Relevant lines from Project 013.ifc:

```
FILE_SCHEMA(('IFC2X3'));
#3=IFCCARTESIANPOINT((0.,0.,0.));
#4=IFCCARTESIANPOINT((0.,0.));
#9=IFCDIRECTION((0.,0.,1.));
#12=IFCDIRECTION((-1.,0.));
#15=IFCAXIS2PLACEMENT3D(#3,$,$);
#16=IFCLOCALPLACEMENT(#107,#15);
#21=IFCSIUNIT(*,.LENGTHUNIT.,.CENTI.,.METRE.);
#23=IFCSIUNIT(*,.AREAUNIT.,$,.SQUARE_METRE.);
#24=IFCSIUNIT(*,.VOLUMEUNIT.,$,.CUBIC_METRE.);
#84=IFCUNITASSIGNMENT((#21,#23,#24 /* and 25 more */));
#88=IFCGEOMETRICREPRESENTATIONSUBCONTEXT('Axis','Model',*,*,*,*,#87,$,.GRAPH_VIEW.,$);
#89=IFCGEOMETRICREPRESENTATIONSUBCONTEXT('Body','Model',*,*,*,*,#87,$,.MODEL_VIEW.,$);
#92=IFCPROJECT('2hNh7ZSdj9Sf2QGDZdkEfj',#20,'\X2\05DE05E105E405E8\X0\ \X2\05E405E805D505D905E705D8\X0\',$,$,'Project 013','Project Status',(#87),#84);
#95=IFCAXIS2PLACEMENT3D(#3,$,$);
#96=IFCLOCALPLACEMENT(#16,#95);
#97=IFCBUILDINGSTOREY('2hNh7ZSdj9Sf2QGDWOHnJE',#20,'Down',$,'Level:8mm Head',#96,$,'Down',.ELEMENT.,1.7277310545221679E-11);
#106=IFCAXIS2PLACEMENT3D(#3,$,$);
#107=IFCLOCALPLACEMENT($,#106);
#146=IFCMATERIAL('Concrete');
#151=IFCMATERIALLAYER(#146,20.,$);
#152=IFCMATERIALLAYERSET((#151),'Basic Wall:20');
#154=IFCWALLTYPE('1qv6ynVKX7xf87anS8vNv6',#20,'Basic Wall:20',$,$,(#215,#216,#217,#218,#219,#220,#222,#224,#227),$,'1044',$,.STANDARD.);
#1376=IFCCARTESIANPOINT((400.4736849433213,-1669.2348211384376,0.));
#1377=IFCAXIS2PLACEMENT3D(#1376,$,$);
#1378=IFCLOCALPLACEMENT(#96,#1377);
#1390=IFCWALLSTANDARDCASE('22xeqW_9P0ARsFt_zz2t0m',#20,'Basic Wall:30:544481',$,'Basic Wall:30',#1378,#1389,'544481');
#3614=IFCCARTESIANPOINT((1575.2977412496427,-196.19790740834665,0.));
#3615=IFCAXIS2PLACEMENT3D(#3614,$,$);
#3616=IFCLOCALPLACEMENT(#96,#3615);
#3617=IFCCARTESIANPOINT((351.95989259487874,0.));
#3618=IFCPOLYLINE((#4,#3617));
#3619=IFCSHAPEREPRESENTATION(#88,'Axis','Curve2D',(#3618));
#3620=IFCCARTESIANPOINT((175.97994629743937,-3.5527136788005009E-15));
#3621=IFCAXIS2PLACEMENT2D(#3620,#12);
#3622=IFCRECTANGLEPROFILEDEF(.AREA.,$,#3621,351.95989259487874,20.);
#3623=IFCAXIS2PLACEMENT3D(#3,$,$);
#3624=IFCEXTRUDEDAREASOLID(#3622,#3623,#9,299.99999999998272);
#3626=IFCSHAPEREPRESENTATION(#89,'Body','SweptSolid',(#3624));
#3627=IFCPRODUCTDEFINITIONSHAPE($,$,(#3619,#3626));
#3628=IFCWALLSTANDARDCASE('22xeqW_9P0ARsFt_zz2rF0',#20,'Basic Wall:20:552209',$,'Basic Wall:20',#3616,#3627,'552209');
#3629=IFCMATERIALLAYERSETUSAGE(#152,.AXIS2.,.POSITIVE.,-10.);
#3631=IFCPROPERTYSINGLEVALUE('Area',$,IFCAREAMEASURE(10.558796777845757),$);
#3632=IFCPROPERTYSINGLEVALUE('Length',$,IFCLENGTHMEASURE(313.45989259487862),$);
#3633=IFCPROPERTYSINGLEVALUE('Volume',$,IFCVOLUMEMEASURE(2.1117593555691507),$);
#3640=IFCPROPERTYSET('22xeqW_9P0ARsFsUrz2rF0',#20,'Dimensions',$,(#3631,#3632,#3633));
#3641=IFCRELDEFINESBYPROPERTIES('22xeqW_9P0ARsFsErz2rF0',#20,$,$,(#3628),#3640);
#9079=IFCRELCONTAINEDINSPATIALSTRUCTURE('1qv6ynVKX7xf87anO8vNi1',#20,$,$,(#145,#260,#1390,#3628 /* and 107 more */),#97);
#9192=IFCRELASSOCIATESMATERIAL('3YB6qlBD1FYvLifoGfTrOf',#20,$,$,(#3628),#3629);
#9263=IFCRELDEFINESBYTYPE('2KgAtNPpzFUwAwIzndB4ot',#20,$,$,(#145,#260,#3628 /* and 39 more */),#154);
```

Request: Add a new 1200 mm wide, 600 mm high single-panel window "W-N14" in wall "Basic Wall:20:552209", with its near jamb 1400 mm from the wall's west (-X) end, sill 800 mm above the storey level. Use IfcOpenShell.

```python
import numpy as np
import ifcopenshell
import ifcopenshell.api.feature
import ifcopenshell.api.geometry
import ifcopenshell.api.pset
import ifcopenshell.api.root
import ifcopenshell.api.spatial
import ifcopenshell.api.type
import ifcopenshell.geom
import ifcopenshell.util.element
import ifcopenshell.util.placement
import ifcopenshell.util.representation
import ifcopenshell.util.shape
import ifcopenshell.util.unit

model = ifcopenshell.open("Project 013.ifc")
unit_scale = ifcopenshell.util.unit.calculate_unit_scale(model)
area_scale = ifcopenshell.util.unit.calculate_unit_scale(model, "AREAUNIT")
volume_scale = ifcopenshell.util.unit.calculate_unit_scale(model, "VOLUMEUNIT")
settings = ifcopenshell.geom.settings()


def volume(element):
    """Net volume in cubic metres, openings subtracted."""
    shape = ifcopenshell.geom.create_shape(settings, element)
    return ifcopenshell.util.shape.get_volume(shape.geometry)


wall = model.by_guid("22xeqW_9P0ARsFt_zz2rF0")
storey = ifcopenshell.util.element.get_container(wall, ifc_class="IfcBuildingStorey")
context = ifcopenshell.util.representation.get_context(model, "Model", "Body", "MODEL_VIEW")
before = volume(wall)

width, height, from_end, sill = 1.2, 0.6, 1.4, 0.8  # metres

# The wall runs along its own X axis, and the end named is its -X end.
wall_shape = ifcopenshell.geom.create_shape(settings, wall)
x, y, z = ifcopenshell.util.shape.get_vertices(wall_shape.geometry).T
start = x.min() + from_end
face, thickness = float(y.min()), float(y.max() - y.min())
wall_matrix = ifcopenshell.util.placement.get_local_placement(wall.ObjectPlacement)
level = ifcopenshell.util.placement.get_local_placement(storey.ObjectPlacement)[2, 3]


def in_wall(x, y):
    """Placement at x, y metres in the wall's axes, at sill height."""
    matrix = wall_matrix.copy()
    matrix[:, 3] = wall_matrix @ np.array([x / unit_scale, y / unit_scale, 0.0, 1.0])
    matrix[2, 3] = level + sill / unit_scale
    return matrix


# Opening: a box that overshoots both wall faces by 50 mm.
opening = ifcopenshell.api.root.create_entity(model, ifc_class="IfcOpeningElement")
box = ifcopenshell.api.geometry.add_wall_representation(
    model, context=context, length=width, height=height, thickness=thickness + 0.1
)
ifcopenshell.api.geometry.assign_representation(model, product=opening, representation=box)
ifcopenshell.api.geometry.edit_object_placement(model, product=opening, matrix=in_wall(start, face - 0.05), is_si=False)
ifcopenshell.api.feature.add_feature(model, feature=opening, element=wall)

window = ifcopenshell.api.root.create_entity(model, ifc_class="IfcWindow", name="W-N14")
window.OverallWidth, window.OverallHeight = width / unit_scale, height / unit_scale
body = ifcopenshell.api.geometry.add_window_representation(
    model,
    context=context,
    overall_width=window.OverallWidth,
    overall_height=window.OverallHeight,
    partition_type="SINGLE_PANEL",
)
ifcopenshell.api.geometry.assign_representation(model, product=window, representation=body)
ifcopenshell.api.spatial.assign_container(model, products=[window], relating_structure=storey)
fills = ifcopenshell.api.feature.add_filling(model, opening=opening, element=window)
fills.OwnerHistory = window.OwnerHistory  # required in IFC2X3

# IFC2X3 keeps the operation on the window style.
style = ifcopenshell.api.root.create_entity(model, ifc_class="IfcWindowStyle", name="W-N14")
style.OperationType, style.ConstructionType = "SINGLE_PANEL", "NOTDEFINED"
style.ParameterTakesPrecedence = style.Sizeable = False
ifcopenshell.api.type.assign_type(model, related_objects=[window], relating_type=style)

# Centre the window in the wall's thickness.
ifcopenshell.api.geometry.edit_object_placement(model, product=window, matrix=in_wall(start, face), is_si=False)
window_shape = ifcopenshell.geom.create_shape(settings, window)
depth = ifcopenshell.util.shape.get_vertices(window_shape.geometry)[:, 1]
offset = face + thickness / 2 - (depth.min() + depth.max()) / 2
ifcopenshell.api.geometry.edit_object_placement(model, product=window, matrix=in_wall(start, offset), is_si=False)

after = volume(wall)

# Update the wall's stored quantities.
pset = model.by_id(ifcopenshell.util.element.get_pset(wall, "Dimensions", should_inherit=False)["id"])
ifcopenshell.api.pset.edit_pset(model, pset=pset, properties={
    "Area": model.create_entity("IfcAreaMeasure", after / thickness / area_scale),
    "Volume": model.create_entity("IfcVolumeMeasure", after / volume_scale),
})

print(f"wall volume {before:.3f} -> {after:.3f} m3")

model.write("Project 013_v2.ifc")
```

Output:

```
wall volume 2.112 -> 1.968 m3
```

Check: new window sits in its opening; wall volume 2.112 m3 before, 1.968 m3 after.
